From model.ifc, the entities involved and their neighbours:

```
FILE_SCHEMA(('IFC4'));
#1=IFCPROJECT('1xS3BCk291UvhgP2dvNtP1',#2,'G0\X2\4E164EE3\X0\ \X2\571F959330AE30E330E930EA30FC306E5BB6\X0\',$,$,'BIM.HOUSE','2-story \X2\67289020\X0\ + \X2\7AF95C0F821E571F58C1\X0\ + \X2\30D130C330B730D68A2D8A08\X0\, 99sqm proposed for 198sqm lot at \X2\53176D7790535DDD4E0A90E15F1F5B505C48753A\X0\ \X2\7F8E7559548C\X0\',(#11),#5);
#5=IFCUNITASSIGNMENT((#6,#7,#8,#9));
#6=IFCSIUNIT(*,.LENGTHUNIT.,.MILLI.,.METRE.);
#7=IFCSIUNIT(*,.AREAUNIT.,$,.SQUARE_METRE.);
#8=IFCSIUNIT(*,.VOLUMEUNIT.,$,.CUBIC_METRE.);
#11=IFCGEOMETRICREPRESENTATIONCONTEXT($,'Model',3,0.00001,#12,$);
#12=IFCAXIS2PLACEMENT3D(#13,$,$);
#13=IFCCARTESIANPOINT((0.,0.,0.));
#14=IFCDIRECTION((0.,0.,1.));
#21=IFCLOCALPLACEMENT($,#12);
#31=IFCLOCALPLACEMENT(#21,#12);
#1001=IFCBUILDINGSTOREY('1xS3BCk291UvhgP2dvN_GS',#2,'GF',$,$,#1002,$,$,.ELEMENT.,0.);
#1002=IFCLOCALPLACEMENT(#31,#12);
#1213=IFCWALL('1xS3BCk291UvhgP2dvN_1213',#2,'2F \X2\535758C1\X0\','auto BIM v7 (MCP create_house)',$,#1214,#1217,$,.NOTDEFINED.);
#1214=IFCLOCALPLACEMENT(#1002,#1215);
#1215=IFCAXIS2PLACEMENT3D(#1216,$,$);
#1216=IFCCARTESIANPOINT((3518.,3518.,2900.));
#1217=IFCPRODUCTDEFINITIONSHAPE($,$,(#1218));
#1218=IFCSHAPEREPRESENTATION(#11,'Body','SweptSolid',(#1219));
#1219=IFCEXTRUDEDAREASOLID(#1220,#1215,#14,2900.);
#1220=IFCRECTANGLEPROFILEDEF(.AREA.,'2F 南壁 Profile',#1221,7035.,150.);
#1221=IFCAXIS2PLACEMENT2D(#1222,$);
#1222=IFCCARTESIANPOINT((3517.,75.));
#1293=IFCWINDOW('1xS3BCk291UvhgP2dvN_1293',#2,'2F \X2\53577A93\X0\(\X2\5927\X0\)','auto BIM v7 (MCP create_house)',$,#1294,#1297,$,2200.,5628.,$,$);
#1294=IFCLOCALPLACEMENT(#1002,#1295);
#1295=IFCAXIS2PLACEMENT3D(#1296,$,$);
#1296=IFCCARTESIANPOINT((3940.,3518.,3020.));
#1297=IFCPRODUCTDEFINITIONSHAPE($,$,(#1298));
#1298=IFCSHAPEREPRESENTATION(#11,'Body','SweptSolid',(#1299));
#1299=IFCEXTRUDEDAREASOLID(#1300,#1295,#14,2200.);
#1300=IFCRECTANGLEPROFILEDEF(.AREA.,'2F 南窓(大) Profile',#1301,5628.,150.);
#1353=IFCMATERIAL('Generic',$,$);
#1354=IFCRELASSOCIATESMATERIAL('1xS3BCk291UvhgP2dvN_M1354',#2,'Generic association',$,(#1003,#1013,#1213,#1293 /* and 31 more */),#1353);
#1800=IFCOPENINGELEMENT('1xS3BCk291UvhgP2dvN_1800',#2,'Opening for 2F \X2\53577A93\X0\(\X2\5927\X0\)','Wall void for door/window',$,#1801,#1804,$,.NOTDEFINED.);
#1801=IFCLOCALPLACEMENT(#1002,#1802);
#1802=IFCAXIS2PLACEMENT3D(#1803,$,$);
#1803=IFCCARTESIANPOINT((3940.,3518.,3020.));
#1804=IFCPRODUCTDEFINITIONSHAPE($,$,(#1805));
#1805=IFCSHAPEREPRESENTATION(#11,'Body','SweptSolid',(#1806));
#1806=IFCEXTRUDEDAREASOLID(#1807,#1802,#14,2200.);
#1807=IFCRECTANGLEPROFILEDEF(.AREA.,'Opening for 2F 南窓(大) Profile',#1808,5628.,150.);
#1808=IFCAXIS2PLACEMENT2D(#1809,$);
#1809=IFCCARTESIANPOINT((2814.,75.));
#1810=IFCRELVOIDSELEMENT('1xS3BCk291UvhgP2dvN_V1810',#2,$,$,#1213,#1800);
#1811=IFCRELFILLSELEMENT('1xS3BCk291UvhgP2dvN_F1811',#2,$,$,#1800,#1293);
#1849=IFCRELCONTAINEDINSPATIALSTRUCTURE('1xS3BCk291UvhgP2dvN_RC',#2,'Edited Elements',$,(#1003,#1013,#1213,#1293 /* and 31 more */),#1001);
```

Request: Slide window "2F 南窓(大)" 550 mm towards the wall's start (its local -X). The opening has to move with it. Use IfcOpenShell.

```python
import ifcopenshell
import ifcopenshell.api.geometry
import ifcopenshell.util.placement

model = ifcopenshell.open("model.ifc")

window = model.by_guid("1xS3BCk291UvhgP2dvN_1293")
opening = window.FillsVoids[0].RelatingOpeningElement
wall = opening.VoidsElements[0].RelatingBuildingElement

wall_matrix = ifcopenshell.util.placement.get_local_placement(wall.ObjectPlacement)
shift = wall_matrix[:3, 0] * -550.0
before = ifcopenshell.util.placement.get_local_placement(window.ObjectPlacement)[:3, 3].copy()

# The window is not placed relative to its opening, so move both.
for product in (opening, window):
    matrix = ifcopenshell.util.placement.get_local_placement(product.ObjectPlacement)
    matrix[:3, 3] += shift
    ifcopenshell.api.geometry.edit_object_placement(model, product=product, matrix=matrix, is_si=False)

after = ifcopenshell.util.placement.get_local_placement(window.ObjectPlacement)[:3, 3]
print("window moved by", (after - before).round(3) + 0.0)

model.write("model_v2.ifc")
```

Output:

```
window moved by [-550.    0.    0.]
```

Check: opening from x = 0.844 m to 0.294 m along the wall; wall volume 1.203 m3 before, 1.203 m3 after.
